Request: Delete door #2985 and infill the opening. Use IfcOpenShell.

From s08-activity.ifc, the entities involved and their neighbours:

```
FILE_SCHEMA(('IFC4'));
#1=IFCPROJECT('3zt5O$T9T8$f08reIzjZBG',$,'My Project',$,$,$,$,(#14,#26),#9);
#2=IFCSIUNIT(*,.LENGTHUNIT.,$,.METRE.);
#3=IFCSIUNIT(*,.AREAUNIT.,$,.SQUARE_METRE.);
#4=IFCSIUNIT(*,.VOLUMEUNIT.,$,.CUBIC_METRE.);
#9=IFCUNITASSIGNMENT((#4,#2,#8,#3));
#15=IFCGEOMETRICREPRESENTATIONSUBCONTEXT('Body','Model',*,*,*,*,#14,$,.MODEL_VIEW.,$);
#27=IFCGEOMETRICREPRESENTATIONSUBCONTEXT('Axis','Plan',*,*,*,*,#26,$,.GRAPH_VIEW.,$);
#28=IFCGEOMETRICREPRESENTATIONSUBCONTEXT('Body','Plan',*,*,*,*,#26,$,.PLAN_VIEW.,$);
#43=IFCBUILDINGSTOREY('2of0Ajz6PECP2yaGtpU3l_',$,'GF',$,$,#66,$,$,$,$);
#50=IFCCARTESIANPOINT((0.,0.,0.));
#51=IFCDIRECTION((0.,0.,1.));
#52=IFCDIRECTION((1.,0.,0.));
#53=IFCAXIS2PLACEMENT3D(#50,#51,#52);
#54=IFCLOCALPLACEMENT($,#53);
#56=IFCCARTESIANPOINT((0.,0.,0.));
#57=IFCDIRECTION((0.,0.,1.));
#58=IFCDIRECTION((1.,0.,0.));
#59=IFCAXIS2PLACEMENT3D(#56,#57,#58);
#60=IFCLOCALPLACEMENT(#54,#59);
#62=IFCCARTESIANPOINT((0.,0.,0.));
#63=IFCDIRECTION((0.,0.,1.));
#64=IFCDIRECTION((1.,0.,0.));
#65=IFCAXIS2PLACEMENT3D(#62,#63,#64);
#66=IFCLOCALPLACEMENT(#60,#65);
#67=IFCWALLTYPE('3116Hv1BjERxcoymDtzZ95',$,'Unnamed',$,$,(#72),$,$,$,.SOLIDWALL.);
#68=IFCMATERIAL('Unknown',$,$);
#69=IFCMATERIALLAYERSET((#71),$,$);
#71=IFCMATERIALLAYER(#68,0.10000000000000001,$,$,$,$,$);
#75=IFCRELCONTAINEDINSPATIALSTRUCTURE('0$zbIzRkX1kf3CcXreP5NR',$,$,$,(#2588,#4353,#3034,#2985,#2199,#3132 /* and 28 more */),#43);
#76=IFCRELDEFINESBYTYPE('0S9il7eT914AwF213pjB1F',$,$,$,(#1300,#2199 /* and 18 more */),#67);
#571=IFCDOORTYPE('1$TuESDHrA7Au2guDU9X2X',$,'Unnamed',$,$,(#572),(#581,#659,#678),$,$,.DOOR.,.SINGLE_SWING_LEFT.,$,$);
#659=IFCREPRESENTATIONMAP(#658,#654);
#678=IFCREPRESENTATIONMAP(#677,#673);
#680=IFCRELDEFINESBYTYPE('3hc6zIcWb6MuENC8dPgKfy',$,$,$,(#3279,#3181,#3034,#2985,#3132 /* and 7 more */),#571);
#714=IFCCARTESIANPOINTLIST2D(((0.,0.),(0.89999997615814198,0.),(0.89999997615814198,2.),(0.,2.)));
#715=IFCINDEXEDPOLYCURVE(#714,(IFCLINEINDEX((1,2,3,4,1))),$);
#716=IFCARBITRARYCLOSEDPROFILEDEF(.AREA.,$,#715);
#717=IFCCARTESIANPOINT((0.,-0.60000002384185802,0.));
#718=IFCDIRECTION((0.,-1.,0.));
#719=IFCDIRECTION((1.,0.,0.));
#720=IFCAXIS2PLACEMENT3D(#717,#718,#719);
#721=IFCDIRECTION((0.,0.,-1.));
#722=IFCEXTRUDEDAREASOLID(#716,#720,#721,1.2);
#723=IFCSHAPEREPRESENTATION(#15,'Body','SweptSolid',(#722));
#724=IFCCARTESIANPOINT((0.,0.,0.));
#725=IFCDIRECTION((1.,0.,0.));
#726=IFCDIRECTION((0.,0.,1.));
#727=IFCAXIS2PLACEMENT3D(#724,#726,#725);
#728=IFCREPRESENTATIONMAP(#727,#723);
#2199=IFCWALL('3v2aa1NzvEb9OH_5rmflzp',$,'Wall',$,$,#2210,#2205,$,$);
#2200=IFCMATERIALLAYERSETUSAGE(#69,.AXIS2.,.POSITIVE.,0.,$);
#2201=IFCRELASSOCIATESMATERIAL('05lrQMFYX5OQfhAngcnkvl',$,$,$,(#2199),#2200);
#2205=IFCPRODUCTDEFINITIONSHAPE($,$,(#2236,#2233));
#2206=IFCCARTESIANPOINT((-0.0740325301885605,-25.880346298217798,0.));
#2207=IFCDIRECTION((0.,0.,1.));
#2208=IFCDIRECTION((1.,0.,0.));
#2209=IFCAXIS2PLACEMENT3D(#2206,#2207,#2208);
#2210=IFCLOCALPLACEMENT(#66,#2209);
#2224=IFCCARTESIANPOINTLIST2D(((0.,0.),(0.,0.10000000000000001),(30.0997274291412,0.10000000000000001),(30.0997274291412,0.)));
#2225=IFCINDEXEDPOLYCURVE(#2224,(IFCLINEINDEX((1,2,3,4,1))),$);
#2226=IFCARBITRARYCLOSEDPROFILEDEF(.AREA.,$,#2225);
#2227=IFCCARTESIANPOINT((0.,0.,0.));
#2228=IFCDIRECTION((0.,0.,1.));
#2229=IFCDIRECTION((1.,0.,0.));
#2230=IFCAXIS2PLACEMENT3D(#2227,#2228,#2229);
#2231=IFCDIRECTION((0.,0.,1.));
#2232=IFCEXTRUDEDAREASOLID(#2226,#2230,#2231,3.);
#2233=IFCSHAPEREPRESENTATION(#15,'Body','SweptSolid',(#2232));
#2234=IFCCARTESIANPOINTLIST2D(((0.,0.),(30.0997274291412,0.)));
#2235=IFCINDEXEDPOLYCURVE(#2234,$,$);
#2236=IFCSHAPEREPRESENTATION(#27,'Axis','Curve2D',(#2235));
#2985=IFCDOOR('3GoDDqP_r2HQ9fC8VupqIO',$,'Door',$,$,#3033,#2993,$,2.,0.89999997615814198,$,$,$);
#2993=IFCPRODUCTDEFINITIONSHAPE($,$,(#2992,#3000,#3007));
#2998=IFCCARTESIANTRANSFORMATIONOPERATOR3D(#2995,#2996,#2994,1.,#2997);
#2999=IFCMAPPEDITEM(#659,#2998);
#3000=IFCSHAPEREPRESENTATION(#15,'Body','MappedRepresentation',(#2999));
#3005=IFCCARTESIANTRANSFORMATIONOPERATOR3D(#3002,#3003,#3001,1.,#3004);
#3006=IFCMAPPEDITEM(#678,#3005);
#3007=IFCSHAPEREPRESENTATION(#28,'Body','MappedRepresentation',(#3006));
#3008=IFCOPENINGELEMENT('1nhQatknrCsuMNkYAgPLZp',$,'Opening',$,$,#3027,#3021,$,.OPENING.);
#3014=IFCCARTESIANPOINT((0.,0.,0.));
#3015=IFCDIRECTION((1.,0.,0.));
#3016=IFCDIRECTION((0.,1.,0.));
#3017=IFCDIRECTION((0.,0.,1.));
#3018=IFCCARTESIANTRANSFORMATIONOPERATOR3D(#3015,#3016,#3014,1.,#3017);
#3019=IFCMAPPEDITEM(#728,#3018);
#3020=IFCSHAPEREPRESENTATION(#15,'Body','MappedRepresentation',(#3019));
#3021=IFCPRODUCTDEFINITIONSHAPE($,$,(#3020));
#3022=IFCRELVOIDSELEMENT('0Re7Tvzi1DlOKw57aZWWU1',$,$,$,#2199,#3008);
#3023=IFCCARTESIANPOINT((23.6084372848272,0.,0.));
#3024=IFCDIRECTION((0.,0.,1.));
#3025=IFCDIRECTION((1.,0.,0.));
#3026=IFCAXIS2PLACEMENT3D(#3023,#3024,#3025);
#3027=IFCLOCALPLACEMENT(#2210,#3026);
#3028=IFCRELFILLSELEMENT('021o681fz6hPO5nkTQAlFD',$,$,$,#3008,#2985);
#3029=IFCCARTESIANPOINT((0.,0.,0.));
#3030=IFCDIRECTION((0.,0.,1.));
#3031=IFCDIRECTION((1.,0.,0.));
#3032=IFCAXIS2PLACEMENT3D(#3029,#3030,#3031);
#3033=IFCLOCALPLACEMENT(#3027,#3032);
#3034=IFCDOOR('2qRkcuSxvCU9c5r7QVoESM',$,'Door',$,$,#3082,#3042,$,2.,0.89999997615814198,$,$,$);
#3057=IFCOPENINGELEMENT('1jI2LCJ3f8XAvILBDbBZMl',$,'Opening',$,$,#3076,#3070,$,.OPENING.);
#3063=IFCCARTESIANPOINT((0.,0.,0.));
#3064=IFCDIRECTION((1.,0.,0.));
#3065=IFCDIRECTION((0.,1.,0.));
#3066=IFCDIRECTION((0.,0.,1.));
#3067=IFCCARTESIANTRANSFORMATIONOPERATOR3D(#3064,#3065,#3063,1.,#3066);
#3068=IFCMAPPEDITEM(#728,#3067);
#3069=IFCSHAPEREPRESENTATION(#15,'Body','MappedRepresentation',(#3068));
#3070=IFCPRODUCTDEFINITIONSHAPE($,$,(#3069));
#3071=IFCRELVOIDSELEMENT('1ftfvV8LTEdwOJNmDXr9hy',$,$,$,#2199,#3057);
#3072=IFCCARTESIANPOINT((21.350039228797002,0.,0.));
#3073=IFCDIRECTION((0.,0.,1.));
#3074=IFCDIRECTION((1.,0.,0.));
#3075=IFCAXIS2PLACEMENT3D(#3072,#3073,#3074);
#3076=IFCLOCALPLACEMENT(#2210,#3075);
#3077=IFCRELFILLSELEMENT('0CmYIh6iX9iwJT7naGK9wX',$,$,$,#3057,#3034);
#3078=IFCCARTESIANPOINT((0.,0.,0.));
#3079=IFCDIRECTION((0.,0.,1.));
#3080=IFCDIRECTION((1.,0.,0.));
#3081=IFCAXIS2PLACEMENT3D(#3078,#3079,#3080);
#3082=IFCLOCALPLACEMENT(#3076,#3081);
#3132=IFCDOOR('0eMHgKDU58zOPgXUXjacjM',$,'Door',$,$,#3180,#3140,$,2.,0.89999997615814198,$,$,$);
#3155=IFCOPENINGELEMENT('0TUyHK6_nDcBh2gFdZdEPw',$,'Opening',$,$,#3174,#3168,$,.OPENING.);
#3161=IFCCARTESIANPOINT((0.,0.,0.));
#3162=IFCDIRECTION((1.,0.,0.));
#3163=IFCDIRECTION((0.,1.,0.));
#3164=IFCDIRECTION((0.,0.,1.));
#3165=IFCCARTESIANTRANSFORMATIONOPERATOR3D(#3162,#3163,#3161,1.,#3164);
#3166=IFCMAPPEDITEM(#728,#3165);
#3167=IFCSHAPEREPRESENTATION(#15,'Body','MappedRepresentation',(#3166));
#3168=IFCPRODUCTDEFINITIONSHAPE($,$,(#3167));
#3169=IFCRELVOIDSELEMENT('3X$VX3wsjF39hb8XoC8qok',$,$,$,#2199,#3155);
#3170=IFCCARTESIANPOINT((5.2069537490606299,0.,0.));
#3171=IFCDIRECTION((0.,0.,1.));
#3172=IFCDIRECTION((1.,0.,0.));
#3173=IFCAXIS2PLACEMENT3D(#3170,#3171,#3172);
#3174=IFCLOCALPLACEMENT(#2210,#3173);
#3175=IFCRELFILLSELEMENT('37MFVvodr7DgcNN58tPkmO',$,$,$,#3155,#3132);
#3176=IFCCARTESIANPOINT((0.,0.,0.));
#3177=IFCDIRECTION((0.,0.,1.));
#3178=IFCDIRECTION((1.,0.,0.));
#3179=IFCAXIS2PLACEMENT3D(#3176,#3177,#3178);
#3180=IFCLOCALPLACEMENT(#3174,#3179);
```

```python
import ifcopenshell
import ifcopenshell.api.feature
import ifcopenshell.api.root
import ifcopenshell.geom
import ifcopenshell.util.shape

model = ifcopenshell.open("s08-activity.ifc")
settings = ifcopenshell.geom.settings()


def volume(element):
    """Net volume in cubic metres, openings subtracted."""
    shape = ifcopenshell.geom.create_shape(settings, element)
    return ifcopenshell.util.shape.get_volume(shape.geometry)


door = model.by_id(2985)
opening = door.FillsVoids[0].RelatingOpeningElement
wall = opening.VoidsElements[0].RelatingBuildingElement
before = volume(wall)

ifcopenshell.api.root.remove_product(model, product=door)
ifcopenshell.api.feature.remove_feature(model, feature=opening)

after = volume(wall)

print(f"wall volume {before:.3f} -> {after:.3f} m3")

model.write("s08-activity_updated.ifc")
```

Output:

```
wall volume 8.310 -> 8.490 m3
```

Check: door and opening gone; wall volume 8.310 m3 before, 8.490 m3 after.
